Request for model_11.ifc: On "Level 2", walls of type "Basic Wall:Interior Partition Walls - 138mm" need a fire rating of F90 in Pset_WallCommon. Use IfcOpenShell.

First a look at what the model holds.

```python
import ifcopenshell
import ifcopenshell.util.element

model = ifcopenshell.open("model_11.ifc")
print(model.schema)
storey = next(s for s in model.by_type("IfcBuildingStorey") if s.Name == "Level 2")
walls = [e for e in ifcopenshell.util.element.get_decomposition(storey) if e.is_a("IfcWall")]
seen = {}
for e in walls:
    element_type = ifcopenshell.util.element.get_type(e)
    key = (element_type.Name if element_type != e and element_type else None, ifcopenshell.util.element.get_pset(e, "Pset_WallCommon", "FireRating"))
    seen[key] = seen.get(key, 0) + 1
for (name, value), count in sorted(seen.items(), key=str):
    print(count, "x", name, "|", value)
```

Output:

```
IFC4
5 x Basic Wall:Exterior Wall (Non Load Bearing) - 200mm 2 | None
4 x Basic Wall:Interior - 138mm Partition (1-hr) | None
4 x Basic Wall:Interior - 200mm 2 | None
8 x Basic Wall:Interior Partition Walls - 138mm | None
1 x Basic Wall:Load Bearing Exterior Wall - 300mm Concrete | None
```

```python
import ifcopenshell
import ifcopenshell.api.pset
import ifcopenshell.util.element

model = ifcopenshell.open("model_11.ifc")

storey = next(s for s in model.by_type("IfcBuildingStorey") if s.Name == "Level 2")
walls = [e for e in ifcopenshell.util.element.get_decomposition(storey) if e.is_a("IfcWall")]

count = 0
for e in walls:
    element_type = ifcopenshell.util.element.get_type(e)
    if element_type in (None, e) or element_type.Name != "Basic Wall:Interior Partition Walls - 138mm":
        continue
    # add_pset returns the element's existing set when there is one.
    pset = ifcopenshell.api.pset.add_pset(model, product=e, name="Pset_WallCommon")
    ifcopenshell.api.pset.edit_pset(model, pset=pset, properties={"FireRating": "F90"})
    count += 1

print(count, "walls updated")

model.write("model_11_v2.ifc")
```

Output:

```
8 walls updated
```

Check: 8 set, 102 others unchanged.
